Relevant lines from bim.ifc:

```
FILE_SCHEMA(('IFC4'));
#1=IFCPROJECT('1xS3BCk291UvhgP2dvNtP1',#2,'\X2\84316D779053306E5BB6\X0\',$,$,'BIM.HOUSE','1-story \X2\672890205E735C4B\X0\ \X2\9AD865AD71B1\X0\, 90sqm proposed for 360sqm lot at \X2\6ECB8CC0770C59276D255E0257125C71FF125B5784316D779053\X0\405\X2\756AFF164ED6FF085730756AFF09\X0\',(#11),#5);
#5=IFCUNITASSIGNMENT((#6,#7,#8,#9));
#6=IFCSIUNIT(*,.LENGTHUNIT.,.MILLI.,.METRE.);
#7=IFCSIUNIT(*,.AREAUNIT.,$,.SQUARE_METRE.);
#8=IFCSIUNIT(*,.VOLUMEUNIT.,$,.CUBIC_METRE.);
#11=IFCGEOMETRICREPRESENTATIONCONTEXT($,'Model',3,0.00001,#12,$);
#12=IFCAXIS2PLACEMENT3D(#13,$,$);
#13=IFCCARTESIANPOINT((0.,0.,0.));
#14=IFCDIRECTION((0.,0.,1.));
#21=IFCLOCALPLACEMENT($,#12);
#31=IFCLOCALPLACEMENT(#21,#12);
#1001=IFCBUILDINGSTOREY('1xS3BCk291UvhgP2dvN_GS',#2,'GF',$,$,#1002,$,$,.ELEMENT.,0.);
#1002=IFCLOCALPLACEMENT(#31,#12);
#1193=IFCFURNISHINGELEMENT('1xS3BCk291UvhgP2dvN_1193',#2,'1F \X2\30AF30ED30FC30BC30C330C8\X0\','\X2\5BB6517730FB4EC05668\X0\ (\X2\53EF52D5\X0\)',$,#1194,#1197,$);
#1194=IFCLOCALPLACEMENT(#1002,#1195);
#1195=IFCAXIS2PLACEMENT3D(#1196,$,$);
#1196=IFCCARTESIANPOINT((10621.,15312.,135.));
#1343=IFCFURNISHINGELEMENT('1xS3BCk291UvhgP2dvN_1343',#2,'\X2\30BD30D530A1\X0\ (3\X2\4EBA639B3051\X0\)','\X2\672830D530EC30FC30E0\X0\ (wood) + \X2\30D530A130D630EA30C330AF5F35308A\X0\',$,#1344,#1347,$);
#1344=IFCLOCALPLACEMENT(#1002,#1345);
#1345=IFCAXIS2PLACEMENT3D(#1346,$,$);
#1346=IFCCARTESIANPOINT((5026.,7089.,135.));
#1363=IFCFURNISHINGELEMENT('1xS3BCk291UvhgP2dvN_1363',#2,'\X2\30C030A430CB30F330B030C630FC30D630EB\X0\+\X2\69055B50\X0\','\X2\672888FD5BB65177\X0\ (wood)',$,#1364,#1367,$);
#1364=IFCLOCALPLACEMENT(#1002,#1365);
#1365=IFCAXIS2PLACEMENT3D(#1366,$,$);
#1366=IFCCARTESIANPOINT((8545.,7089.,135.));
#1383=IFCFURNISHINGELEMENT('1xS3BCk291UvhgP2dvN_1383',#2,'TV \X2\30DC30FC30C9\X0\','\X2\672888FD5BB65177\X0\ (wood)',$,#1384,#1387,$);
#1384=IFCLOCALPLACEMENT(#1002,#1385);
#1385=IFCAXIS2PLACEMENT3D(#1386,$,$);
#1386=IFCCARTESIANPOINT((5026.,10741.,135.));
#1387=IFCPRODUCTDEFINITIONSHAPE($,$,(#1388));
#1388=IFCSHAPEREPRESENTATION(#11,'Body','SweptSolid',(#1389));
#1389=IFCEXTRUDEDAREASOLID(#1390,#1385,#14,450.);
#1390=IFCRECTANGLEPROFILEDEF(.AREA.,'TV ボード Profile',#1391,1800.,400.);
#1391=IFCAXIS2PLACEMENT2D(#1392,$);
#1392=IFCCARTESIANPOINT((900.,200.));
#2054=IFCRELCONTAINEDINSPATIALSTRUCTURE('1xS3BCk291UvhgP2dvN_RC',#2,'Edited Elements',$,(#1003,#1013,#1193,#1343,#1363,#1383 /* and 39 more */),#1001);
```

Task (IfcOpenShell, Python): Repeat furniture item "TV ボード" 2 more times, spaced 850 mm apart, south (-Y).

```python
import numpy as np
import ifcopenshell
import ifcopenshell.api.geometry
import ifcopenshell.api.root
import ifcopenshell.util.element
import ifcopenshell.util.placement

model = ifcopenshell.open("bim.ifc")


def reuse_history(source, copy):
    """copy_class also copies each property set's owner history, people and application; keep the originals."""
    for rel in copy.IsDefinedBy:
        if rel.is_a("IfcRelDefinesByProperties") and (history := rel.RelatingPropertyDefinition.OwnerHistory):
            rel.RelatingPropertyDefinition.OwnerHistory = source.OwnerHistory
            ifcopenshell.util.element.remove_deep2(model, history)


source = model.by_guid("1xS3BCk291UvhgP2dvN_1383")
base = ifcopenshell.util.placement.get_local_placement(source.ObjectPlacement)
step = np.array([0.0, -1.0, 0.0]) * 850.0

for i in range(1, 3):
    copy = ifcopenshell.api.root.copy_class(model, product=source)
    copy.Representation = ifcopenshell.util.element.copy_deep(
        model, source.Representation, exclude=["IfcGeometricRepresentationContext", "IfcRepresentationMap"]
    )
    reuse_history(source, copy)
    matrix = base.copy()
    matrix[:3, 3] += i * step
    print("added at", matrix[:3, 3].round(3) + 0.0)
    ifcopenshell.api.geometry.edit_object_placement(model, product=copy, matrix=matrix, is_si=False)

model.write("bim_v2.ifc")
```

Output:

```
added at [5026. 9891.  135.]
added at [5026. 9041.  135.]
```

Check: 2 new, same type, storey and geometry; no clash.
